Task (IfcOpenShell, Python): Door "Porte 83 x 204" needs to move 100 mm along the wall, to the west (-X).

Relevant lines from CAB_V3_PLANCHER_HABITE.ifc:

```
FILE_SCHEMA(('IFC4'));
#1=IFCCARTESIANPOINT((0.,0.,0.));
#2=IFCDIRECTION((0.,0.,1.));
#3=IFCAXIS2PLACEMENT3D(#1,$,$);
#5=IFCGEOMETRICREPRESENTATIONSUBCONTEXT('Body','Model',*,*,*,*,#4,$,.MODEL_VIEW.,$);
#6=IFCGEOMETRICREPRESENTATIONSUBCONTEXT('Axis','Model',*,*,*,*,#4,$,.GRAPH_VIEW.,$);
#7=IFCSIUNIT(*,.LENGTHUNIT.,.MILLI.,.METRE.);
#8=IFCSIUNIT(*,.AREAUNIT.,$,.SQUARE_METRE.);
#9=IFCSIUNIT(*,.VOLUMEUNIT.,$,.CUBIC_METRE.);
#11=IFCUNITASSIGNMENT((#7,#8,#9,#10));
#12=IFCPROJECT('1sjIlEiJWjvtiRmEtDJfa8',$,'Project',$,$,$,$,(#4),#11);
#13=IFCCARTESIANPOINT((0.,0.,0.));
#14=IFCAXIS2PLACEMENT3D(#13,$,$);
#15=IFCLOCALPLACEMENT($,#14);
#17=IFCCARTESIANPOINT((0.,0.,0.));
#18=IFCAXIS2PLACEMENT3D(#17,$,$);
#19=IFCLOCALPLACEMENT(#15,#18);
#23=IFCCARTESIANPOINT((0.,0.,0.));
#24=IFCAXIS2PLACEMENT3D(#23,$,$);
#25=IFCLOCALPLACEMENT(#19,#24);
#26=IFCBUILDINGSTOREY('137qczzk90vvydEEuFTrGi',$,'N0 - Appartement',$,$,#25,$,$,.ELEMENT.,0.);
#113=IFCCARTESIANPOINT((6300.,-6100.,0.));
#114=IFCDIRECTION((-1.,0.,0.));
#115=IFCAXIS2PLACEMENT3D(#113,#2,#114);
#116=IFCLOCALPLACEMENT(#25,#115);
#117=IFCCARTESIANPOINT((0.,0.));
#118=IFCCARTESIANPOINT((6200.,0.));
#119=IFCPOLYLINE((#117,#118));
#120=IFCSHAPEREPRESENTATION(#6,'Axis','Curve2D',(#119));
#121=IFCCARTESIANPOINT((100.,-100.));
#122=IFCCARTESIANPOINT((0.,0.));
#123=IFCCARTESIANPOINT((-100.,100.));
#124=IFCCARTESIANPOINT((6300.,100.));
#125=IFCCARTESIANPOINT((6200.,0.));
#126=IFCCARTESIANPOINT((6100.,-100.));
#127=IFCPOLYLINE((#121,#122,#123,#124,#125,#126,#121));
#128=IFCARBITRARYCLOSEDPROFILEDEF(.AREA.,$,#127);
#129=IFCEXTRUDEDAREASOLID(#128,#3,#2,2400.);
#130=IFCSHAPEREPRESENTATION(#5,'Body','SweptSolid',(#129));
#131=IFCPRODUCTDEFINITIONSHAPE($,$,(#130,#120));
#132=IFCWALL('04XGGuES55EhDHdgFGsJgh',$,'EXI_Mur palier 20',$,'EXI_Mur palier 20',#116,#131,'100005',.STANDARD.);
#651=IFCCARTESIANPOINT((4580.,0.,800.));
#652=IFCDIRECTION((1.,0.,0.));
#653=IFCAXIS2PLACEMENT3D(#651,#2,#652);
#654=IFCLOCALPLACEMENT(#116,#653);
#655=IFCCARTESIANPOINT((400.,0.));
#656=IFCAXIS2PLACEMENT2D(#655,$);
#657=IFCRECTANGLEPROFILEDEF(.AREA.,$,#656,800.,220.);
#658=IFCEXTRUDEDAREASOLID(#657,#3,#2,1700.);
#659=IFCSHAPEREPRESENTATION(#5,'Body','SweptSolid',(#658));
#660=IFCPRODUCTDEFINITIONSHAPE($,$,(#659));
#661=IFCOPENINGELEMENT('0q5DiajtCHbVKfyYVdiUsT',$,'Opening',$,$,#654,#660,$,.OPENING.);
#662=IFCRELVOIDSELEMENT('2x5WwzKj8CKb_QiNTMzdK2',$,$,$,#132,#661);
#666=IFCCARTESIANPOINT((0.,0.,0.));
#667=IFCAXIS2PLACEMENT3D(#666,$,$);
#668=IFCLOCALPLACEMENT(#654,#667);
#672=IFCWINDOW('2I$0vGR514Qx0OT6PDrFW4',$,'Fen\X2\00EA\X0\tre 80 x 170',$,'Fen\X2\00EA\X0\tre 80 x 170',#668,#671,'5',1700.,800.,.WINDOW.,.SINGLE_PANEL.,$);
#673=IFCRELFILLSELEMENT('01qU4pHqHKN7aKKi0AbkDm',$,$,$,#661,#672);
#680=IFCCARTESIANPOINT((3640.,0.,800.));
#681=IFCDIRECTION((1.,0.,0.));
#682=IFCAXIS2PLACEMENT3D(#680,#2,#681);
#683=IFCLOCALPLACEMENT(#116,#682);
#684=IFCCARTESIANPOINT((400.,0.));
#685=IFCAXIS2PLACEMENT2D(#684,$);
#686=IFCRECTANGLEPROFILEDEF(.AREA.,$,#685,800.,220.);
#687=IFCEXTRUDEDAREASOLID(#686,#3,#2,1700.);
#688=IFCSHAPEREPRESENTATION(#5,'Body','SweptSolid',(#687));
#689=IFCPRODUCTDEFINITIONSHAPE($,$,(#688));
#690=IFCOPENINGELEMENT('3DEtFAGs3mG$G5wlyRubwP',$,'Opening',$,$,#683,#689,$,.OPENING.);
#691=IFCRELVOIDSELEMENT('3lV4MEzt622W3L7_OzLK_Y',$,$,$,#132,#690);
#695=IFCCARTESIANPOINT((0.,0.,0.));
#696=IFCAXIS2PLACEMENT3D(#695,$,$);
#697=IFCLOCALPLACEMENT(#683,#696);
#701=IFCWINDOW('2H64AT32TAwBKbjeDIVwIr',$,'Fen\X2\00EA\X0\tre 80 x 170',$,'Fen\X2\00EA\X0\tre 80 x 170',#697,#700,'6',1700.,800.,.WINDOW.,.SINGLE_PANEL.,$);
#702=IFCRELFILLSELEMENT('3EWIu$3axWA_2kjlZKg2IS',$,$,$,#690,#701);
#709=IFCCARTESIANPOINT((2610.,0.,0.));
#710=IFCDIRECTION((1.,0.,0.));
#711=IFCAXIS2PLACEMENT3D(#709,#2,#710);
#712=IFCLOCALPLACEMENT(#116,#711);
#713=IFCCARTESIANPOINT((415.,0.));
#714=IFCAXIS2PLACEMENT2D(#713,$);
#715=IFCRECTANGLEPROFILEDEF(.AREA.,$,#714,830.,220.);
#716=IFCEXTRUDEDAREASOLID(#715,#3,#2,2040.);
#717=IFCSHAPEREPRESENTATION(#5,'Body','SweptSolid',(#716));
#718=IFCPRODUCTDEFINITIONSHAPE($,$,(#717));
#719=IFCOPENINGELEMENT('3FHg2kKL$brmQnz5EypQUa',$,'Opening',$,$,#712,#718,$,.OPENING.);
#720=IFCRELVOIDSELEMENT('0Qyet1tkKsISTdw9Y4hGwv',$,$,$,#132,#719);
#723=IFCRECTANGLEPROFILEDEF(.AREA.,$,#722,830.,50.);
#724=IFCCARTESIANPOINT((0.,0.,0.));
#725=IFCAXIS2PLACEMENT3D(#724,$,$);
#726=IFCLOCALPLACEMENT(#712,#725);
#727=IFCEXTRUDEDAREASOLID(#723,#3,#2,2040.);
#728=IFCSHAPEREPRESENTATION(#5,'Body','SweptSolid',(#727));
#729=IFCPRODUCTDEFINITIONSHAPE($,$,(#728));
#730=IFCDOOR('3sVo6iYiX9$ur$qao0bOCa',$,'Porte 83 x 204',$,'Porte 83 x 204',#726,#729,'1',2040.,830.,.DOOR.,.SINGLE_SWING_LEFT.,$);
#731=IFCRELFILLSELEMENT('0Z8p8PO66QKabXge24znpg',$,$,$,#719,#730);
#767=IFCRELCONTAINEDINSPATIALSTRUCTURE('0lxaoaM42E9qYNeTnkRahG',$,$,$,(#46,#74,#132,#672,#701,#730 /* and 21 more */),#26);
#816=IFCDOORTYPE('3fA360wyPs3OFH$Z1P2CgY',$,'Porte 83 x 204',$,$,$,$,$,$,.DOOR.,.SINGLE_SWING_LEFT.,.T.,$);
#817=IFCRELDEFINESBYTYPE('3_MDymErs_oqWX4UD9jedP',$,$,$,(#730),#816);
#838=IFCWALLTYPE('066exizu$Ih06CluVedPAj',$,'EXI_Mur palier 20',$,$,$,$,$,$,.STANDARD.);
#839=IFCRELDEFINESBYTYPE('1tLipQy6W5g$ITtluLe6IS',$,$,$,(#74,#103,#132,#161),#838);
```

```python
import ifcopenshell
import ifcopenshell.api.geometry
import ifcopenshell.util.placement

model = ifcopenshell.open("CAB_V3_PLANCHER_HABITE.ifc")

door = model.by_guid("3sVo6iYiX9$ur$qao0bOCa")
opening = door.FillsVoids[0].RelatingOpeningElement
wall = opening.VoidsElements[0].RelatingBuildingElement

wall_matrix = ifcopenshell.util.placement.get_local_placement(wall.ObjectPlacement)
shift = wall_matrix[:3, 0] * 100.0
before = ifcopenshell.util.placement.get_local_placement(door.ObjectPlacement)[:3, 3].copy()

# The door is placed relative to its opening, so it follows when the opening moves.
matrix = ifcopenshell.util.placement.get_local_placement(opening.ObjectPlacement)
matrix[:3, 3] += shift
ifcopenshell.api.geometry.edit_object_placement(
    model, product=opening, matrix=matrix, is_si=False, should_transform_children=True
)

after = ifcopenshell.util.placement.get_local_placement(door.ObjectPlacement)[:3, 3]
print("door moved by", (after - before).round(3) + 0.0)

model.write("CAB_V3_PLANCHER_HABITE_edited.ifc")
```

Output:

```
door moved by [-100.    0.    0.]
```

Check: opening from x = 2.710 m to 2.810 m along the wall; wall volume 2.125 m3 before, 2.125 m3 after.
